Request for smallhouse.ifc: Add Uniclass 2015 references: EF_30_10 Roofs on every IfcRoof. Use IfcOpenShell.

First a look at what the model holds.

```python
import ifcopenshell

model = ifcopenshell.open("smallhouse.ifc")
print(model.schema)
print("classifications:", [c.Name for c in model.by_type("IfcClassification")])
for ifc_class in ("IfcDoor", "IfcRoof", "IfcStair", "IfcWall", "IfcWindow"):
    print(ifc_class, len(model.by_type(ifc_class)))
```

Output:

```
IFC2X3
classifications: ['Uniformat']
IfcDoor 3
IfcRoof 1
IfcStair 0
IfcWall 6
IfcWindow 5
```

```python
import ifcopenshell
import ifcopenshell.api.classification

model = ifcopenshell.open("smallhouse.ifc")

# IFC2X3 requires Source and Edition and has no link from the project to the system.
system = model.create_entity("IfcClassification", Source="NBS", Edition="2015", Name="Uniclass 2015")

codes = {
    "IfcRoof": ("EF_30_10", "Roofs"),
}
for ifc_class, (code, name) in codes.items():
    products = model.by_type(ifc_class)
    ifcopenshell.api.classification.add_reference(
        model, products=products, classification=system, identification=code, name=name
    )
    print(code, len(products))

model.write("smallhouse_v2.ifc")
```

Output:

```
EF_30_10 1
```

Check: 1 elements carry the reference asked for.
